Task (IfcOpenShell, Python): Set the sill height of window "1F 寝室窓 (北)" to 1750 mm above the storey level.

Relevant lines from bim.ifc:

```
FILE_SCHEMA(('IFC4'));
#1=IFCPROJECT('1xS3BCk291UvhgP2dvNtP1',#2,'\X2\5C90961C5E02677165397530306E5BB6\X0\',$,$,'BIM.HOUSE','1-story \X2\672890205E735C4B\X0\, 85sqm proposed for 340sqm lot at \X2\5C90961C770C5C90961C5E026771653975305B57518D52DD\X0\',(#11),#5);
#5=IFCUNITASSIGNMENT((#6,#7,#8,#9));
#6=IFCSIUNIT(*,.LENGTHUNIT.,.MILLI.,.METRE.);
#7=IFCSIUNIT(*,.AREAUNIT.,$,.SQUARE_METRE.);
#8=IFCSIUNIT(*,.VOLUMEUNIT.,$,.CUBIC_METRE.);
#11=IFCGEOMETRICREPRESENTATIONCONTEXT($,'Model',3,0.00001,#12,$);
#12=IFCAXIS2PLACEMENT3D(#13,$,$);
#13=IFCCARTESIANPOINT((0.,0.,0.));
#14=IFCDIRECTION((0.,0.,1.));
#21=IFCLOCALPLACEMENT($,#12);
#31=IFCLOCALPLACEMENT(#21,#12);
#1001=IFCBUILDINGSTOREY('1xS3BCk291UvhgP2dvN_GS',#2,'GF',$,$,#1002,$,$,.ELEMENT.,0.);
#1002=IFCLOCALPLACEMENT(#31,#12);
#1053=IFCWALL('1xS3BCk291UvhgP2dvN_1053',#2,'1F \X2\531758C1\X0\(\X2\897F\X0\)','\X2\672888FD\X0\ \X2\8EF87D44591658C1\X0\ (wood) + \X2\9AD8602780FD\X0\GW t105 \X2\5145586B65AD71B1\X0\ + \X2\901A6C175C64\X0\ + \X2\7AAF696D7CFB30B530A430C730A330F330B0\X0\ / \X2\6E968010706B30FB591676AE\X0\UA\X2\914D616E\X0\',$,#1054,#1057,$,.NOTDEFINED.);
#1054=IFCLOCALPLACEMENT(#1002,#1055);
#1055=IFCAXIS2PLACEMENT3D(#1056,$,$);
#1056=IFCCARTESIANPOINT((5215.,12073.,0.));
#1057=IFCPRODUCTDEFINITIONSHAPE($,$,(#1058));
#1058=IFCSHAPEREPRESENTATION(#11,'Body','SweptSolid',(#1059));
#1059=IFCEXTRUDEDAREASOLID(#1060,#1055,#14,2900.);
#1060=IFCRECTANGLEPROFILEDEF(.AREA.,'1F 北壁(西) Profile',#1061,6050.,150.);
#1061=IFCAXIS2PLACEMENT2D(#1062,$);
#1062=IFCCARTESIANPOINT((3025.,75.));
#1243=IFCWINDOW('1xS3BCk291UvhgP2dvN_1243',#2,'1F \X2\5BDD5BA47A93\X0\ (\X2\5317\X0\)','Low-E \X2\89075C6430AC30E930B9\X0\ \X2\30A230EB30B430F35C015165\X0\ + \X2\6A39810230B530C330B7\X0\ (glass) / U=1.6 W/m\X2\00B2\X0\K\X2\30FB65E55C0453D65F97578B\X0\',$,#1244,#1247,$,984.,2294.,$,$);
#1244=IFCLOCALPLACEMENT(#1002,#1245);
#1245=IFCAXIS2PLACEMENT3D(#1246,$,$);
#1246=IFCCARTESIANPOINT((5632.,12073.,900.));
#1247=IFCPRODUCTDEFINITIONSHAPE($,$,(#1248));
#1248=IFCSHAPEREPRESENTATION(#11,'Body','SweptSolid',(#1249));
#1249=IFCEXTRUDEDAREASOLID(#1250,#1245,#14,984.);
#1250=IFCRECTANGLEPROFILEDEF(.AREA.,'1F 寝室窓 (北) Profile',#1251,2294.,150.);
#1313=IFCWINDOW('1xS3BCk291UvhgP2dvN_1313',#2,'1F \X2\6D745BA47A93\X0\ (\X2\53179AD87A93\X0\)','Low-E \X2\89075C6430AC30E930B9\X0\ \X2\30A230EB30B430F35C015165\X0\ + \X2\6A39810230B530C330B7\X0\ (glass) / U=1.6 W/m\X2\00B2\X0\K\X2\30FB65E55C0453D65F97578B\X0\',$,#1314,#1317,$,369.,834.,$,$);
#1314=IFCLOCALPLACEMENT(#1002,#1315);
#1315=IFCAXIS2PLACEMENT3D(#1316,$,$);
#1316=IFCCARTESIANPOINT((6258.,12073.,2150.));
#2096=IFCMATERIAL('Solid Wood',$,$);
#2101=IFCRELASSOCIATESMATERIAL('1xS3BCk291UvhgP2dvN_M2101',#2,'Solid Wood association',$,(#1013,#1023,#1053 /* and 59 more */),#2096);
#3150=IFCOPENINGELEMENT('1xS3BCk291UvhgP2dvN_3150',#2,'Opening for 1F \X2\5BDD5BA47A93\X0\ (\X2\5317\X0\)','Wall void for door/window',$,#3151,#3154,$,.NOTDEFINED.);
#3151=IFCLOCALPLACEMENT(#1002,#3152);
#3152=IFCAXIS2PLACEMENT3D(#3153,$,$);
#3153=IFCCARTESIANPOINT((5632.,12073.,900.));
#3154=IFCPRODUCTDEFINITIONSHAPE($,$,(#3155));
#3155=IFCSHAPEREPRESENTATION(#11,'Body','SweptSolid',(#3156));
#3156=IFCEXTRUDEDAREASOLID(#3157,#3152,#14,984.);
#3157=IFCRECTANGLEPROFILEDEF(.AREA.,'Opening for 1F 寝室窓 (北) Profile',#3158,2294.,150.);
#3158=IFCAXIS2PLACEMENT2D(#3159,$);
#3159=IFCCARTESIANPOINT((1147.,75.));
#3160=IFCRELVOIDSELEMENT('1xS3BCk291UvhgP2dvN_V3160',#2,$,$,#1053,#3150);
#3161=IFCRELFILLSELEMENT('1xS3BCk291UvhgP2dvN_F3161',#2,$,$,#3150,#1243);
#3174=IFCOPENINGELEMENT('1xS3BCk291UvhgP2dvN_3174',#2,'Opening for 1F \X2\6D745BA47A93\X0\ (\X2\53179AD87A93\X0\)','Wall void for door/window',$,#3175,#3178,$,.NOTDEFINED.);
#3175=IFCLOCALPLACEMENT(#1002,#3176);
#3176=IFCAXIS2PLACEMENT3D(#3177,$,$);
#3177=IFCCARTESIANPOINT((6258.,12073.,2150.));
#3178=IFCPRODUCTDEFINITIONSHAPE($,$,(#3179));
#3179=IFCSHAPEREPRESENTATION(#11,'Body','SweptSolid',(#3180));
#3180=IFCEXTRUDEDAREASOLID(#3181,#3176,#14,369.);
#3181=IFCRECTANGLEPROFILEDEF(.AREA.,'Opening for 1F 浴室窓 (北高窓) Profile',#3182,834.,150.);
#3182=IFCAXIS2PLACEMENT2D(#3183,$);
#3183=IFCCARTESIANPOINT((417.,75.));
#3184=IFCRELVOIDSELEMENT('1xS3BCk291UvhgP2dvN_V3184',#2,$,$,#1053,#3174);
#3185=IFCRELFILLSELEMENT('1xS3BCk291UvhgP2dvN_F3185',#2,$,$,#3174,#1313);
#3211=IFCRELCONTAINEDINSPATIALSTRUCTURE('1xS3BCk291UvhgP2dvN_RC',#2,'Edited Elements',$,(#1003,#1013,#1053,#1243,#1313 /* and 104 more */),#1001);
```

```python
import numpy as np
import ifcopenshell
import ifcopenshell.api.geometry
import ifcopenshell.geom
import ifcopenshell.util.element
import ifcopenshell.util.placement
import ifcopenshell.util.shape
import ifcopenshell.util.unit

model = ifcopenshell.open("bim.ifc")
unit_scale = ifcopenshell.util.unit.calculate_unit_scale(model)

window = model.by_id(1243)
opening = window.FillsVoids[0].RelatingOpeningElement
storey = ifcopenshell.util.element.get_container(window, ifc_class="IfcBuildingStorey")
level = ifcopenshell.util.placement.get_local_placement(storey.ObjectPlacement)[2, 3]

# The opening's origin need not be at the sill, so measure its lowest point.
shape = ifcopenshell.geom.create_shape(ifcopenshell.geom.settings(), opening)
bottom = ifcopenshell.util.shape.get_shape_bottom_elevation(shape, shape.geometry) / unit_scale
dz = level + 1.75 / unit_scale - bottom

shift = np.array([0.0, 0.0, dz])
# The window is not placed relative to its opening, so move both.
for product in (opening, window):
    matrix = ifcopenshell.util.placement.get_local_placement(product.ObjectPlacement)
    matrix[:3, 3] += shift
    ifcopenshell.api.geometry.edit_object_placement(model, product=product, matrix=matrix, is_si=False)

print(f"moved by {dz * unit_scale:+.3f} m")

model.write("bim_v2.ifc")
```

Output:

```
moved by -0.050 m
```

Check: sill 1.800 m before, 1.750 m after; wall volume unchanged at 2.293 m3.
